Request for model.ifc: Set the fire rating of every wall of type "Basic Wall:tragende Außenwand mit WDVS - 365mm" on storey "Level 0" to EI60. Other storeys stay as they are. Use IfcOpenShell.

First a look at what the model holds.

```python
import ifcopenshell
import ifcopenshell.util.element

model = ifcopenshell.open("model.ifc")
print(model.schema)
storey = next(s for s in model.by_type("IfcBuildingStorey") if s.Name == "Level 0")
walls = [e for e in ifcopenshell.util.element.get_decomposition(storey) if e.is_a("IfcWall")]
seen = {}
for e in walls:
    element_type = ifcopenshell.util.element.get_type(e)
    key = (element_type.Name if element_type != e and element_type else None, ifcopenshell.util.element.get_pset(e, "Pset_WallCommon", "FireRating"))
    seen[key] = seen.get(key, 0) + 1
for (name, value), count in sorted(seen.items(), key=str):
    print(count, "x", name, "|", value)
```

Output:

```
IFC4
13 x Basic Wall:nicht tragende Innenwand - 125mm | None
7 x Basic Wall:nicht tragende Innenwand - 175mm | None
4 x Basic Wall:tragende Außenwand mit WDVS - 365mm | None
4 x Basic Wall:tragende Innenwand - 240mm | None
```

```python
import ifcopenshell
import ifcopenshell.api.pset
import ifcopenshell.util.element

model = ifcopenshell.open("model.ifc")

storey = next(s for s in model.by_type("IfcBuildingStorey") if s.Name == "Level 0")
walls = [e for e in ifcopenshell.util.element.get_decomposition(storey) if e.is_a("IfcWall")]

count = 0
for e in walls:
    element_type = ifcopenshell.util.element.get_type(e)
    if element_type in (None, e) or element_type.Name != "Basic Wall:tragende Außenwand mit WDVS - 365mm":
        continue
    # add_pset returns the element's existing set when there is one.
    pset = ifcopenshell.api.pset.add_pset(model, product=e, name="Pset_WallCommon")
    ifcopenshell.api.pset.edit_pset(model, pset=pset, properties={"FireRating": "EI60"})
    count += 1

print(count, "walls updated")

model.write("model_updated.ifc")
```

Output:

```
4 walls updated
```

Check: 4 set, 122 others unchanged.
